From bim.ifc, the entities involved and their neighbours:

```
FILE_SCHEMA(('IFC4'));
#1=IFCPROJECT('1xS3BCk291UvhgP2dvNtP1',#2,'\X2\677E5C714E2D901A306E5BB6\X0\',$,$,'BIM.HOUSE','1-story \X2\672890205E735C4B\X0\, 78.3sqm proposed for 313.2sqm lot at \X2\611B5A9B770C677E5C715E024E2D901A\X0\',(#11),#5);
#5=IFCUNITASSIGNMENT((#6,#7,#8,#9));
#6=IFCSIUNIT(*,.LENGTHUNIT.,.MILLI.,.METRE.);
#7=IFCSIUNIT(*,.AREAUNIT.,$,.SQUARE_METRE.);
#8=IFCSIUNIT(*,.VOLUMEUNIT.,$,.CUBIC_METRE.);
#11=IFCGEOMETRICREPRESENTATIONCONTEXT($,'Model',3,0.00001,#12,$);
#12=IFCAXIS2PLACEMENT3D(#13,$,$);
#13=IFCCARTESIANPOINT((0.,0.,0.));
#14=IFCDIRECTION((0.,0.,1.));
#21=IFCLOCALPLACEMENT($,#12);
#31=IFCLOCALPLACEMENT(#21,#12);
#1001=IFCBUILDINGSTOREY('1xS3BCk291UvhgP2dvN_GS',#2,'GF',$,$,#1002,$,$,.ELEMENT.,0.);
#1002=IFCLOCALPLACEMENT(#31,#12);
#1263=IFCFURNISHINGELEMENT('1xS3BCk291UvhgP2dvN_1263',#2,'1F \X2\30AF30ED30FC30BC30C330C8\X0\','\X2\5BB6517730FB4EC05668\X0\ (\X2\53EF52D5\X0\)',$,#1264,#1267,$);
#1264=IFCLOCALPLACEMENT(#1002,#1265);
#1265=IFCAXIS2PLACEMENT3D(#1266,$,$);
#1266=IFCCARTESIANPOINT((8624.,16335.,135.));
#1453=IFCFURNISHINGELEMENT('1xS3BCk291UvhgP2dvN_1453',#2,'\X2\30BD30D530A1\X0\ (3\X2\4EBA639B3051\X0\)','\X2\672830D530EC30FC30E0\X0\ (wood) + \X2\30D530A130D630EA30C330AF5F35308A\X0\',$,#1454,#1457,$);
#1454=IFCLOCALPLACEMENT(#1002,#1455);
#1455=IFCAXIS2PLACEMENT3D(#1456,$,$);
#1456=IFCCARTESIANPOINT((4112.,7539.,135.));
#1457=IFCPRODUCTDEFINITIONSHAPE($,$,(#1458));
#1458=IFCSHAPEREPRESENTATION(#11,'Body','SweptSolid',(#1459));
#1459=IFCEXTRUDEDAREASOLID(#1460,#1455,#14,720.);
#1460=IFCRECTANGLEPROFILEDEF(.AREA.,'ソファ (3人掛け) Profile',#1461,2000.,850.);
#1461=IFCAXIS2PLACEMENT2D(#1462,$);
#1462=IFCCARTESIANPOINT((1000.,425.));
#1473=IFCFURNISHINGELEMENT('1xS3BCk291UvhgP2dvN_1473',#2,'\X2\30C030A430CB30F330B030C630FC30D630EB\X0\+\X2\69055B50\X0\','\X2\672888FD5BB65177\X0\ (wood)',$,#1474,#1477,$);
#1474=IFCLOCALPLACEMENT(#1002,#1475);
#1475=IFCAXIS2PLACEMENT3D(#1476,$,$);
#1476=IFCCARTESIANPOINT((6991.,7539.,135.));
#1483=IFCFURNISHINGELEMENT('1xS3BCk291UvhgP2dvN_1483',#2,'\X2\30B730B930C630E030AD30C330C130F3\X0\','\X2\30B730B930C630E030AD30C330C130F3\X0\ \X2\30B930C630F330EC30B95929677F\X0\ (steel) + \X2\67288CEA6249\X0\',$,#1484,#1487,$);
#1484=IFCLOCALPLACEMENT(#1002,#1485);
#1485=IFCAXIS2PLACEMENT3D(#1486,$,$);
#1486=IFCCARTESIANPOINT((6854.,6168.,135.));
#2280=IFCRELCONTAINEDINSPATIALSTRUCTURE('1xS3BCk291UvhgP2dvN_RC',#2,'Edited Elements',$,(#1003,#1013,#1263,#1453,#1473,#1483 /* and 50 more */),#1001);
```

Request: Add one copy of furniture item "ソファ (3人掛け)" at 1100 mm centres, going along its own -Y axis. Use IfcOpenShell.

```python
import ifcopenshell
import ifcopenshell.api.geometry
import ifcopenshell.api.root
import ifcopenshell.util.element
import ifcopenshell.util.placement
import ifcopenshell.util.unit

model = ifcopenshell.open("bim.ifc")
unit_scale = ifcopenshell.util.unit.calculate_unit_scale(model)


def reuse_history(source, copy):
    """copy_class also copies each property set's owner history, people and application; keep the originals."""
    for rel in copy.IsDefinedBy:
        if rel.is_a("IfcRelDefinesByProperties") and (history := rel.RelatingPropertyDefinition.OwnerHistory):
            rel.RelatingPropertyDefinition.OwnerHistory = source.OwnerHistory
            ifcopenshell.util.element.remove_deep2(model, history)


source = model.by_guid("1xS3BCk291UvhgP2dvN_1453")
base = ifcopenshell.util.placement.get_local_placement(source.ObjectPlacement)
step = -base[:3, 1] * 1.1 / unit_scale

for i in range(1, 2):
    copy = ifcopenshell.api.root.copy_class(model, product=source)
    copy.Representation = ifcopenshell.util.element.copy_deep(
        model, source.Representation, exclude=["IfcGeometricRepresentationContext", "IfcRepresentationMap"]
    )
    reuse_history(source, copy)
    matrix = base.copy()
    matrix[:3, 3] += i * step
    print("added at", matrix[:3, 3].round(3) + 0.0)
    ifcopenshell.api.geometry.edit_object_placement(model, product=copy, matrix=matrix, is_si=False)

model.write("bim_updated.ifc")
```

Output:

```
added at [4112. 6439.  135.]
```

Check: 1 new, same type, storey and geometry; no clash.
